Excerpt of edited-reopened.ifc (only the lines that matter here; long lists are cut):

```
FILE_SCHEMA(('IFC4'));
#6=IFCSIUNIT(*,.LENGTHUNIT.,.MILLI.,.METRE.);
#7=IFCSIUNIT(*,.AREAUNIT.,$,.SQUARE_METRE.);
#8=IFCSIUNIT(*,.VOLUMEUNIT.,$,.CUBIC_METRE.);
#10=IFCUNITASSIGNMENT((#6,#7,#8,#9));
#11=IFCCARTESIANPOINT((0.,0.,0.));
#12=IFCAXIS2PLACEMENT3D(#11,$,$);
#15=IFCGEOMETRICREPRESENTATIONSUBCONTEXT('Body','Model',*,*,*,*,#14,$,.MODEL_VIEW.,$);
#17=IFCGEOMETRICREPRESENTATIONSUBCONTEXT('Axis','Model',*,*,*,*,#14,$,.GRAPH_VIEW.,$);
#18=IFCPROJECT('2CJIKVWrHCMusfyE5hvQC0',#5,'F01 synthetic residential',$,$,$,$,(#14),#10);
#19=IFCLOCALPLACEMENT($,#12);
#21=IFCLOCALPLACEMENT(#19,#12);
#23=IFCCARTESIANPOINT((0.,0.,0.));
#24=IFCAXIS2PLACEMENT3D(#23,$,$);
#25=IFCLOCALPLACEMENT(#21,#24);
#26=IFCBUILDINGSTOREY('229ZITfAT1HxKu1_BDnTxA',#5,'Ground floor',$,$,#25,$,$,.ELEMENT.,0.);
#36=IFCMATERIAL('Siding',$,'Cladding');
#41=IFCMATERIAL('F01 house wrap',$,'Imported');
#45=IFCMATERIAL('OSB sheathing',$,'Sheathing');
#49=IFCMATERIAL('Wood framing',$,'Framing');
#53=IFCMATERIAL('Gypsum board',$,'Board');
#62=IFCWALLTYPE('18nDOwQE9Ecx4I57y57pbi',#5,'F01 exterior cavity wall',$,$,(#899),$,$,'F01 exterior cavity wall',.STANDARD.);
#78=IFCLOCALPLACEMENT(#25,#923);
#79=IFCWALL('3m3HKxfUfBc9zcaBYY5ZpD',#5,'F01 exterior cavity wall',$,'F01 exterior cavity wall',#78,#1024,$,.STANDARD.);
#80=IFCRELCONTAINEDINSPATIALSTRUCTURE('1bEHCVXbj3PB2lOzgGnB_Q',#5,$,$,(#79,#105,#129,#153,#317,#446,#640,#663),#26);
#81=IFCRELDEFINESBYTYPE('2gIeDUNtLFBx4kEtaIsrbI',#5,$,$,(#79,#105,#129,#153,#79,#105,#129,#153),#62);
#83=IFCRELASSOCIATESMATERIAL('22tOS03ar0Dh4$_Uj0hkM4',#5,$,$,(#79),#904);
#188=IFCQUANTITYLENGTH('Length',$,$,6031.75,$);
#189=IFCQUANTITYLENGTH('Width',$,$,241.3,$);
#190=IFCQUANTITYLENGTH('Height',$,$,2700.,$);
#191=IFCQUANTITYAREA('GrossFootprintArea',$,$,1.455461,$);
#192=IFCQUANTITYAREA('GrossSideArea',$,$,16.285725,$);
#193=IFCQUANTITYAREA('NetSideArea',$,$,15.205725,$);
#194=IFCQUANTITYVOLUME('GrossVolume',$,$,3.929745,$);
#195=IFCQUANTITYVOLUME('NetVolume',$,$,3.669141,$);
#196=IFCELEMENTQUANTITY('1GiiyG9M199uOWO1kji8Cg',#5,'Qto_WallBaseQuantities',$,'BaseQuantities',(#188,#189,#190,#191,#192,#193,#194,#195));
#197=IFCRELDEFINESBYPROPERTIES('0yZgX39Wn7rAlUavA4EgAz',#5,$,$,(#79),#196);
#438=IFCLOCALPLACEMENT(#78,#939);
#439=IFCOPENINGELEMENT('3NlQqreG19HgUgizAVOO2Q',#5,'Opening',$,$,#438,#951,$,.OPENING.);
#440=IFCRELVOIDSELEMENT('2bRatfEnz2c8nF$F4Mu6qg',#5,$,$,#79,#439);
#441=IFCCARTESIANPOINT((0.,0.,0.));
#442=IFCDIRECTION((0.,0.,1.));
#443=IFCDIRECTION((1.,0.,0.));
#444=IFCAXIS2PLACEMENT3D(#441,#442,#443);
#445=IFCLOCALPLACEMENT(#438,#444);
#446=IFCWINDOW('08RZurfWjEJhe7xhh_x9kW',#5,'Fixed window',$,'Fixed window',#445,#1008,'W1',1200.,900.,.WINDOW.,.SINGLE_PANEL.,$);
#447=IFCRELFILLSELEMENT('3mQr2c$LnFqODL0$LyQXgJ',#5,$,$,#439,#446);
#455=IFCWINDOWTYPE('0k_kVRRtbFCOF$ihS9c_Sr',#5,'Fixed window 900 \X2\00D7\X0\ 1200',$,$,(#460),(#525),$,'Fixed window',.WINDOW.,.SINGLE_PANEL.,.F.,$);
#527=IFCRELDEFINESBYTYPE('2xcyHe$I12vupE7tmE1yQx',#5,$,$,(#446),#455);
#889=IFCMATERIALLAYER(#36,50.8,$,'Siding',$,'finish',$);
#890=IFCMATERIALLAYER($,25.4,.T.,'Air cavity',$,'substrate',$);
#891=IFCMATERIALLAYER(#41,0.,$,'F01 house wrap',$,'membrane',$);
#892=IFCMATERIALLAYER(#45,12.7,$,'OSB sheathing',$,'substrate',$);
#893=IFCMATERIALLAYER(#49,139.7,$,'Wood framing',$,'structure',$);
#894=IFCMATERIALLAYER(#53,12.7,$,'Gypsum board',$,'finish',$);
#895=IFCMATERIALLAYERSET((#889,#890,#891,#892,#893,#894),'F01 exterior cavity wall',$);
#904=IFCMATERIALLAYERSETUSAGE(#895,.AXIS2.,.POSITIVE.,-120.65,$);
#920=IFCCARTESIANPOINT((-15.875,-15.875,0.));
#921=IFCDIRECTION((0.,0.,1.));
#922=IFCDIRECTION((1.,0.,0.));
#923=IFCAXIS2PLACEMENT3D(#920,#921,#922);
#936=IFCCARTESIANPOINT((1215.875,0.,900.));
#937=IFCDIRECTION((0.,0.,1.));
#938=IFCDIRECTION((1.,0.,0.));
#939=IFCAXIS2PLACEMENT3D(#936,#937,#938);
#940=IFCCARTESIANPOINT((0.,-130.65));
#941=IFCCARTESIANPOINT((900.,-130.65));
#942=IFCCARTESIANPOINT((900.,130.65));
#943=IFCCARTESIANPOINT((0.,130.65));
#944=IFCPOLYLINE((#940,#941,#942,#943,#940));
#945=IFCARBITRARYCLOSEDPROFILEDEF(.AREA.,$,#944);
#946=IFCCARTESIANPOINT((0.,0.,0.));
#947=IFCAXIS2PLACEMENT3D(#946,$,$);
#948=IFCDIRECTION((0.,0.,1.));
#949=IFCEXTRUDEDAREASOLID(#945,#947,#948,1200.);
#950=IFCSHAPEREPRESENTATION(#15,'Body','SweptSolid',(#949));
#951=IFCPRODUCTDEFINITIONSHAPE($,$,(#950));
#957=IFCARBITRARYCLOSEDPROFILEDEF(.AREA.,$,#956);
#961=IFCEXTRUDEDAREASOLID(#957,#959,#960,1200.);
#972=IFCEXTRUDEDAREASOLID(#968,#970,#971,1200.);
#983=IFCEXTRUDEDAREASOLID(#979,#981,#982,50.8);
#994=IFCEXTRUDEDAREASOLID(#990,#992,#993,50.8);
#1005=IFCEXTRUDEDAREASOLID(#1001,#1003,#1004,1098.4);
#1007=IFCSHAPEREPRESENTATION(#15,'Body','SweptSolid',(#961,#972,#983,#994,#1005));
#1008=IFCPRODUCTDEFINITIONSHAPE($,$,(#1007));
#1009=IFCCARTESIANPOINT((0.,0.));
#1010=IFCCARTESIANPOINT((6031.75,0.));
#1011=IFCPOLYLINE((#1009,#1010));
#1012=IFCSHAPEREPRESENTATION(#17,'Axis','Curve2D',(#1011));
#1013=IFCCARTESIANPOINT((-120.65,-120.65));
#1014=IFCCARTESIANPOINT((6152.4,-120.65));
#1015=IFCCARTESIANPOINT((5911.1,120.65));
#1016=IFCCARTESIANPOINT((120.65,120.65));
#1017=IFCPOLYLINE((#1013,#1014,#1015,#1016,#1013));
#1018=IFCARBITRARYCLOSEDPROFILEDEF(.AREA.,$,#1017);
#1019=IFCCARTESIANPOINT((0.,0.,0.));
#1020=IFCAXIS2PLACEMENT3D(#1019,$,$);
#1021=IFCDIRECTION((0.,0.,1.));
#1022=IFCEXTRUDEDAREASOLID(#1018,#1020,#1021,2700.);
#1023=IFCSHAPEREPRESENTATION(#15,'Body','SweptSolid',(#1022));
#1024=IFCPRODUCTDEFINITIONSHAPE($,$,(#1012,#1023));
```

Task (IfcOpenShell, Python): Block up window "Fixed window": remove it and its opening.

```python
import ifcopenshell
import ifcopenshell.api.feature
import ifcopenshell.api.pset
import ifcopenshell.api.root
import ifcopenshell.geom
import ifcopenshell.util.element
import ifcopenshell.util.shape
import ifcopenshell.util.unit

model = ifcopenshell.open("edited-reopened.ifc")
area_scale = ifcopenshell.util.unit.calculate_unit_scale(model, "AREAUNIT")
volume_scale = ifcopenshell.util.unit.calculate_unit_scale(model, "VOLUMEUNIT")
settings = ifcopenshell.geom.settings()


def volume(element):
    """Net volume in cubic metres, openings subtracted."""
    shape = ifcopenshell.geom.create_shape(settings, element)
    return ifcopenshell.util.shape.get_volume(shape.geometry)


window = model.by_guid("08RZurfWjEJhe7xhh_x9kW")
opening = window.FillsVoids[0].RelatingOpeningElement
wall = opening.VoidsElements[0].RelatingBuildingElement
before = volume(wall)

ifcopenshell.api.root.remove_product(model, product=window)
ifcopenshell.api.feature.remove_feature(model, feature=opening)

after = volume(wall)
thickness = 0.2413  # wall thickness in metres

# Update the wall's stored quantities.
qto = model.by_id(ifcopenshell.util.element.get_pset(wall, "Qto_WallBaseQuantities", should_inherit=False)["id"])
ifcopenshell.api.pset.edit_qto(model, qto=qto, properties={
    "NetSideArea": after / thickness / area_scale,
    "NetVolume": after / volume_scale,
})

print(f"wall volume {before:.3f} -> {after:.3f} m3")

model.write("edited-reopened_v2.ifc")
```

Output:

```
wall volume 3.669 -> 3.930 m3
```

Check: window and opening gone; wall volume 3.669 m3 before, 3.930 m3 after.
